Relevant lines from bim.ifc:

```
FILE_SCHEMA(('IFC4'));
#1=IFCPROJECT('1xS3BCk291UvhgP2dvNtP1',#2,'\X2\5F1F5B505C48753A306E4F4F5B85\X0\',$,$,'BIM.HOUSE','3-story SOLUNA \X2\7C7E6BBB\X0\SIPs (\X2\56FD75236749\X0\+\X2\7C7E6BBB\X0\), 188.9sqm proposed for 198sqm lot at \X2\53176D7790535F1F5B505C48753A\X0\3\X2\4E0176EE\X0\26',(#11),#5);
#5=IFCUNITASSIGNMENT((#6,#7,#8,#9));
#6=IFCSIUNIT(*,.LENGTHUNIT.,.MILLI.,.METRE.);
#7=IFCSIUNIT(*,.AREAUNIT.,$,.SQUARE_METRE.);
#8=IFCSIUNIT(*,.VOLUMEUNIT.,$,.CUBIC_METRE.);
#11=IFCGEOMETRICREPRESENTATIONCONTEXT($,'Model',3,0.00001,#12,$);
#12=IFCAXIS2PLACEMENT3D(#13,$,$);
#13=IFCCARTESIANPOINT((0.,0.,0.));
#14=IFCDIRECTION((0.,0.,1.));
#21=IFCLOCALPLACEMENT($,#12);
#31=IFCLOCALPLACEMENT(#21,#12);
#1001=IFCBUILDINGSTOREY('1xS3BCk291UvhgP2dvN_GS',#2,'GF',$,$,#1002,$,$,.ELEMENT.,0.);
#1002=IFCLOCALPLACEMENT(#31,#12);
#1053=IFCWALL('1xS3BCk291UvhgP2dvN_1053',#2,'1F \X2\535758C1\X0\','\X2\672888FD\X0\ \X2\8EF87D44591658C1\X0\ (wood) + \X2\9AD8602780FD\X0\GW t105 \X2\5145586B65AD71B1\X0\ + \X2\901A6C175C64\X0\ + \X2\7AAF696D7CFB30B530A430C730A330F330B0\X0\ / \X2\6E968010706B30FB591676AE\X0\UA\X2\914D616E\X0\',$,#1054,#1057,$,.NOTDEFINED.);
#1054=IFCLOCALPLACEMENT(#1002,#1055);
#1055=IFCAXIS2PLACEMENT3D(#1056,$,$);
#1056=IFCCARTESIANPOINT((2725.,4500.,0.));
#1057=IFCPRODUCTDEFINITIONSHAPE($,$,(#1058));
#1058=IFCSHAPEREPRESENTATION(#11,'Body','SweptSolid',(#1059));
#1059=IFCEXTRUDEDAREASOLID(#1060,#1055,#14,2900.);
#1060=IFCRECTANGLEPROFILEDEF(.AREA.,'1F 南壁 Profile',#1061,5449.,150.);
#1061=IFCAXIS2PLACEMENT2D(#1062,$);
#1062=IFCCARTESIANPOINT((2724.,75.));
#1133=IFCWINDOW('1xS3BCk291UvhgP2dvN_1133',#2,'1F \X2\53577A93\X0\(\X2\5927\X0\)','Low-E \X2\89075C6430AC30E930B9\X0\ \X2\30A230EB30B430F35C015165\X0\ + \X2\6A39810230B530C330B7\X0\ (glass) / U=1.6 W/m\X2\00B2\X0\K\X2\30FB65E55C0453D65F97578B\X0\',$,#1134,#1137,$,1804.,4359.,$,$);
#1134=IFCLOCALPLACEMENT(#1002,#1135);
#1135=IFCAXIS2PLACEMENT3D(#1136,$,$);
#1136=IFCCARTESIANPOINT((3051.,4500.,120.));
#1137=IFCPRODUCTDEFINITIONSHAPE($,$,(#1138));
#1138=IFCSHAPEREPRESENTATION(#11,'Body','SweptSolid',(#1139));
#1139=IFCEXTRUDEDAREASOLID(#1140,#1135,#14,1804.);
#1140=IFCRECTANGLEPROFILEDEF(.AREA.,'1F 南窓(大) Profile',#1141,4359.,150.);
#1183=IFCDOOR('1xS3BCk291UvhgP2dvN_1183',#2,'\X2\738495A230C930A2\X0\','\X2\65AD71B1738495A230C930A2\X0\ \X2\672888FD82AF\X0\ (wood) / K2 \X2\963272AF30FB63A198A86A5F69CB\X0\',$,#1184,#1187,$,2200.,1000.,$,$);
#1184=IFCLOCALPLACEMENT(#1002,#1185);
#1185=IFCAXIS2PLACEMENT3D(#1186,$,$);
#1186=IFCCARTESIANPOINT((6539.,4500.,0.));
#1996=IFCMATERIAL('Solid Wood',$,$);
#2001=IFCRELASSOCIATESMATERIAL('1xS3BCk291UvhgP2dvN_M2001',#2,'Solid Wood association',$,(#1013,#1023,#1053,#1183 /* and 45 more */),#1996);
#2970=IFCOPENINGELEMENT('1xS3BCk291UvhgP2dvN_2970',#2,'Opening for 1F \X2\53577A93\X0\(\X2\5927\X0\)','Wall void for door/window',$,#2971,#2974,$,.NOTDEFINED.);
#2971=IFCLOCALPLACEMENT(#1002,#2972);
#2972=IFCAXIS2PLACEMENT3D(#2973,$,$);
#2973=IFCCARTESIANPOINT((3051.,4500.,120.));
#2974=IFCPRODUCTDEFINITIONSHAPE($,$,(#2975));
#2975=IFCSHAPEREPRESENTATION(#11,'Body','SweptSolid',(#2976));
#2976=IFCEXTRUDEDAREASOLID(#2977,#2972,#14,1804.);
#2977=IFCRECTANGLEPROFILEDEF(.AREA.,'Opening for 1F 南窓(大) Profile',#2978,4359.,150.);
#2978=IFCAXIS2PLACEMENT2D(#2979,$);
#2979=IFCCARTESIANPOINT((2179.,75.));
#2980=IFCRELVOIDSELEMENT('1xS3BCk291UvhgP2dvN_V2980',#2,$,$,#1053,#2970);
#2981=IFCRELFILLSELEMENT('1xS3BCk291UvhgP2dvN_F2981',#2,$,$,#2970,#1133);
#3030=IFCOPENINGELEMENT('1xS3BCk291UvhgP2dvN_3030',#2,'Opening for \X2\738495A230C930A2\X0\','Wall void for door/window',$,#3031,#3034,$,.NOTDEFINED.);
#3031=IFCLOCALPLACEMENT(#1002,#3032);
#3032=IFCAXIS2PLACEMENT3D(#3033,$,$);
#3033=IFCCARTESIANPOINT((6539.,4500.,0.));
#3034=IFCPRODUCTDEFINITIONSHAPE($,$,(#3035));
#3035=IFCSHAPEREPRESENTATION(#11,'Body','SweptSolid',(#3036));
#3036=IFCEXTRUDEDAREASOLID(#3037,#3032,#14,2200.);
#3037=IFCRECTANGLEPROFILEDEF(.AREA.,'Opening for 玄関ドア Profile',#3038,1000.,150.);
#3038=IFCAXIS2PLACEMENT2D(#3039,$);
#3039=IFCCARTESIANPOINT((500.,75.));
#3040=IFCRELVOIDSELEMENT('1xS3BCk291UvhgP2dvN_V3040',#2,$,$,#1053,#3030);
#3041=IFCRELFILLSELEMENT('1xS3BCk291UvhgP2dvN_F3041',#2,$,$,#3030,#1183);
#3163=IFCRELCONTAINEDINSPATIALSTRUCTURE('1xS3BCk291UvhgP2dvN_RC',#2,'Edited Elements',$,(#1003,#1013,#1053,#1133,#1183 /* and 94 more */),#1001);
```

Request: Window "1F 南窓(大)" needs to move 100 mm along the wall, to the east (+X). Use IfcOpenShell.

```python
import ifcopenshell
import ifcopenshell.api.geometry
import ifcopenshell.util.placement
import ifcopenshell.util.unit

model = ifcopenshell.open("bim.ifc")
unit_scale = ifcopenshell.util.unit.calculate_unit_scale(model)

window = model.by_guid("1xS3BCk291UvhgP2dvN_1133")
opening = window.FillsVoids[0].RelatingOpeningElement
wall = opening.VoidsElements[0].RelatingBuildingElement

wall_matrix = ifcopenshell.util.placement.get_local_placement(wall.ObjectPlacement)
shift = wall_matrix[:3, 0] * 0.1 / unit_scale
before = ifcopenshell.util.placement.get_local_placement(window.ObjectPlacement)[:3, 3].copy()

# The window is not placed relative to its opening, so move both.
for product in (opening, window):
    matrix = ifcopenshell.util.placement.get_local_placement(product.ObjectPlacement)
    matrix[:3, 3] += shift
    ifcopenshell.api.geometry.edit_object_placement(model, product=product, matrix=matrix, is_si=False)

after = ifcopenshell.util.placement.get_local_placement(window.ObjectPlacement)[:3, 3]
print("window moved by", (after - before).round(3) + 0.0)

model.write("bim_updated.ifc")
```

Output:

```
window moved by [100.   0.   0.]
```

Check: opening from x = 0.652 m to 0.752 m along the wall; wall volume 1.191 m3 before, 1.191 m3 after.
